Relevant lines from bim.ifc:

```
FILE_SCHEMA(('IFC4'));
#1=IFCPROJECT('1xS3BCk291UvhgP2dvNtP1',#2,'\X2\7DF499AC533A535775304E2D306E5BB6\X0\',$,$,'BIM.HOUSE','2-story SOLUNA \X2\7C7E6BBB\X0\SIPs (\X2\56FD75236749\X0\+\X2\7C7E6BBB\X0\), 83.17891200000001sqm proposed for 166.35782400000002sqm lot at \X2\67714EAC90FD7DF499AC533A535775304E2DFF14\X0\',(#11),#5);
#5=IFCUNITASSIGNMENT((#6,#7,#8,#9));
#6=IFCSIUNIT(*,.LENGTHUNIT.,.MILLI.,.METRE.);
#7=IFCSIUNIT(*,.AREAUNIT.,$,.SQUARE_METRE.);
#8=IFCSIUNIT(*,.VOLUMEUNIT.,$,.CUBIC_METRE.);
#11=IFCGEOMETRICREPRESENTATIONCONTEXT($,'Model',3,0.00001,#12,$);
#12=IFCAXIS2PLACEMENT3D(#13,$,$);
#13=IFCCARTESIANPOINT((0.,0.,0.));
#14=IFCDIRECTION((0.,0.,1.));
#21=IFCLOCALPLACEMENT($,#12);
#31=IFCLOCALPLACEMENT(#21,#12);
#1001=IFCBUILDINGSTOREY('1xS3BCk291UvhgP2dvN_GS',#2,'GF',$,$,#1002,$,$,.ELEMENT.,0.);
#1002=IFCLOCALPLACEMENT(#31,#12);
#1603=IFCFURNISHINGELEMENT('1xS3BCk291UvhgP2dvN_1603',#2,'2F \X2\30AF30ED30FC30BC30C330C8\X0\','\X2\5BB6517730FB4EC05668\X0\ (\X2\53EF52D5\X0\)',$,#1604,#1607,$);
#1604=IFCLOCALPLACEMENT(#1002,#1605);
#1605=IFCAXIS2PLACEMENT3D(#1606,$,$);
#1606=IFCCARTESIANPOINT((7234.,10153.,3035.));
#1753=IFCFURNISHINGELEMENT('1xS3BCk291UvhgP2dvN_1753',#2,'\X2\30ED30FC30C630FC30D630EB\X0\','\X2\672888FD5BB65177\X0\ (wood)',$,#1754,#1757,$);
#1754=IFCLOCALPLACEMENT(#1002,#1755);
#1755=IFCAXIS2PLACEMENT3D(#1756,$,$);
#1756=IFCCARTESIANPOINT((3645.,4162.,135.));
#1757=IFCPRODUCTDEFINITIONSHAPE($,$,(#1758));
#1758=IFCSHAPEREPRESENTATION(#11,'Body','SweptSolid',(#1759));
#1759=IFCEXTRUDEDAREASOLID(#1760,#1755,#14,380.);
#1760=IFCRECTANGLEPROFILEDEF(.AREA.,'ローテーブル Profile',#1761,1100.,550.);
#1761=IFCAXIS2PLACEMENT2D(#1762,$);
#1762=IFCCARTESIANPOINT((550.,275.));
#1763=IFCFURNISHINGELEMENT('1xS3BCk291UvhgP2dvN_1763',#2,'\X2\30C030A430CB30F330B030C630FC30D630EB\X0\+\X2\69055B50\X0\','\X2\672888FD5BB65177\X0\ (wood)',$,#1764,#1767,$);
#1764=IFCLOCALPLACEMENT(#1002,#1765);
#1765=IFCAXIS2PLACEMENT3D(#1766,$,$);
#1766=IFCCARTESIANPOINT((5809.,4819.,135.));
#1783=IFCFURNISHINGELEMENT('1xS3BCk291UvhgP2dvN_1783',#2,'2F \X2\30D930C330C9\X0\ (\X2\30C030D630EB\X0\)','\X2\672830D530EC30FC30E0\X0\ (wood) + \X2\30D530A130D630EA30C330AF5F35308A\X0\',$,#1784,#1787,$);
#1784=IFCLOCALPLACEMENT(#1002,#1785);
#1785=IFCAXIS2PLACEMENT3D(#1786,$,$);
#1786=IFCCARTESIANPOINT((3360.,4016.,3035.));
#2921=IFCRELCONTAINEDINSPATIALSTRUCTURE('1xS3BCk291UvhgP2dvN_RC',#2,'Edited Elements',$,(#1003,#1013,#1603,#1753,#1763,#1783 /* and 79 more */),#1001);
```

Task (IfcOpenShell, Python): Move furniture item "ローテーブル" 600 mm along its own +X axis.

```python
import ifcopenshell
import ifcopenshell.api.geometry
import ifcopenshell.util.placement
import ifcopenshell.util.unit

model = ifcopenshell.open("bim.ifc")
unit_scale = ifcopenshell.util.unit.calculate_unit_scale(model)

item = model.by_id(1753)
matrix = ifcopenshell.util.placement.get_local_placement(item.ObjectPlacement)
matrix[:3, 3] += matrix[:3, 0] * 0.6 / unit_scale
ifcopenshell.api.geometry.edit_object_placement(model, product=item, matrix=matrix, is_si=False)

print(ifcopenshell.util.placement.get_local_placement(item.ObjectPlacement).round(3) + 0.0)

model.write("bim_edited.ifc")
```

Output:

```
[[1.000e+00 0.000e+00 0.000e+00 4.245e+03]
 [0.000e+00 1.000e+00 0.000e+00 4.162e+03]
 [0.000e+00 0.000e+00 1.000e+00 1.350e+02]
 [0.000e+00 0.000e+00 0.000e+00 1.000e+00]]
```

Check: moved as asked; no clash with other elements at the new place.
